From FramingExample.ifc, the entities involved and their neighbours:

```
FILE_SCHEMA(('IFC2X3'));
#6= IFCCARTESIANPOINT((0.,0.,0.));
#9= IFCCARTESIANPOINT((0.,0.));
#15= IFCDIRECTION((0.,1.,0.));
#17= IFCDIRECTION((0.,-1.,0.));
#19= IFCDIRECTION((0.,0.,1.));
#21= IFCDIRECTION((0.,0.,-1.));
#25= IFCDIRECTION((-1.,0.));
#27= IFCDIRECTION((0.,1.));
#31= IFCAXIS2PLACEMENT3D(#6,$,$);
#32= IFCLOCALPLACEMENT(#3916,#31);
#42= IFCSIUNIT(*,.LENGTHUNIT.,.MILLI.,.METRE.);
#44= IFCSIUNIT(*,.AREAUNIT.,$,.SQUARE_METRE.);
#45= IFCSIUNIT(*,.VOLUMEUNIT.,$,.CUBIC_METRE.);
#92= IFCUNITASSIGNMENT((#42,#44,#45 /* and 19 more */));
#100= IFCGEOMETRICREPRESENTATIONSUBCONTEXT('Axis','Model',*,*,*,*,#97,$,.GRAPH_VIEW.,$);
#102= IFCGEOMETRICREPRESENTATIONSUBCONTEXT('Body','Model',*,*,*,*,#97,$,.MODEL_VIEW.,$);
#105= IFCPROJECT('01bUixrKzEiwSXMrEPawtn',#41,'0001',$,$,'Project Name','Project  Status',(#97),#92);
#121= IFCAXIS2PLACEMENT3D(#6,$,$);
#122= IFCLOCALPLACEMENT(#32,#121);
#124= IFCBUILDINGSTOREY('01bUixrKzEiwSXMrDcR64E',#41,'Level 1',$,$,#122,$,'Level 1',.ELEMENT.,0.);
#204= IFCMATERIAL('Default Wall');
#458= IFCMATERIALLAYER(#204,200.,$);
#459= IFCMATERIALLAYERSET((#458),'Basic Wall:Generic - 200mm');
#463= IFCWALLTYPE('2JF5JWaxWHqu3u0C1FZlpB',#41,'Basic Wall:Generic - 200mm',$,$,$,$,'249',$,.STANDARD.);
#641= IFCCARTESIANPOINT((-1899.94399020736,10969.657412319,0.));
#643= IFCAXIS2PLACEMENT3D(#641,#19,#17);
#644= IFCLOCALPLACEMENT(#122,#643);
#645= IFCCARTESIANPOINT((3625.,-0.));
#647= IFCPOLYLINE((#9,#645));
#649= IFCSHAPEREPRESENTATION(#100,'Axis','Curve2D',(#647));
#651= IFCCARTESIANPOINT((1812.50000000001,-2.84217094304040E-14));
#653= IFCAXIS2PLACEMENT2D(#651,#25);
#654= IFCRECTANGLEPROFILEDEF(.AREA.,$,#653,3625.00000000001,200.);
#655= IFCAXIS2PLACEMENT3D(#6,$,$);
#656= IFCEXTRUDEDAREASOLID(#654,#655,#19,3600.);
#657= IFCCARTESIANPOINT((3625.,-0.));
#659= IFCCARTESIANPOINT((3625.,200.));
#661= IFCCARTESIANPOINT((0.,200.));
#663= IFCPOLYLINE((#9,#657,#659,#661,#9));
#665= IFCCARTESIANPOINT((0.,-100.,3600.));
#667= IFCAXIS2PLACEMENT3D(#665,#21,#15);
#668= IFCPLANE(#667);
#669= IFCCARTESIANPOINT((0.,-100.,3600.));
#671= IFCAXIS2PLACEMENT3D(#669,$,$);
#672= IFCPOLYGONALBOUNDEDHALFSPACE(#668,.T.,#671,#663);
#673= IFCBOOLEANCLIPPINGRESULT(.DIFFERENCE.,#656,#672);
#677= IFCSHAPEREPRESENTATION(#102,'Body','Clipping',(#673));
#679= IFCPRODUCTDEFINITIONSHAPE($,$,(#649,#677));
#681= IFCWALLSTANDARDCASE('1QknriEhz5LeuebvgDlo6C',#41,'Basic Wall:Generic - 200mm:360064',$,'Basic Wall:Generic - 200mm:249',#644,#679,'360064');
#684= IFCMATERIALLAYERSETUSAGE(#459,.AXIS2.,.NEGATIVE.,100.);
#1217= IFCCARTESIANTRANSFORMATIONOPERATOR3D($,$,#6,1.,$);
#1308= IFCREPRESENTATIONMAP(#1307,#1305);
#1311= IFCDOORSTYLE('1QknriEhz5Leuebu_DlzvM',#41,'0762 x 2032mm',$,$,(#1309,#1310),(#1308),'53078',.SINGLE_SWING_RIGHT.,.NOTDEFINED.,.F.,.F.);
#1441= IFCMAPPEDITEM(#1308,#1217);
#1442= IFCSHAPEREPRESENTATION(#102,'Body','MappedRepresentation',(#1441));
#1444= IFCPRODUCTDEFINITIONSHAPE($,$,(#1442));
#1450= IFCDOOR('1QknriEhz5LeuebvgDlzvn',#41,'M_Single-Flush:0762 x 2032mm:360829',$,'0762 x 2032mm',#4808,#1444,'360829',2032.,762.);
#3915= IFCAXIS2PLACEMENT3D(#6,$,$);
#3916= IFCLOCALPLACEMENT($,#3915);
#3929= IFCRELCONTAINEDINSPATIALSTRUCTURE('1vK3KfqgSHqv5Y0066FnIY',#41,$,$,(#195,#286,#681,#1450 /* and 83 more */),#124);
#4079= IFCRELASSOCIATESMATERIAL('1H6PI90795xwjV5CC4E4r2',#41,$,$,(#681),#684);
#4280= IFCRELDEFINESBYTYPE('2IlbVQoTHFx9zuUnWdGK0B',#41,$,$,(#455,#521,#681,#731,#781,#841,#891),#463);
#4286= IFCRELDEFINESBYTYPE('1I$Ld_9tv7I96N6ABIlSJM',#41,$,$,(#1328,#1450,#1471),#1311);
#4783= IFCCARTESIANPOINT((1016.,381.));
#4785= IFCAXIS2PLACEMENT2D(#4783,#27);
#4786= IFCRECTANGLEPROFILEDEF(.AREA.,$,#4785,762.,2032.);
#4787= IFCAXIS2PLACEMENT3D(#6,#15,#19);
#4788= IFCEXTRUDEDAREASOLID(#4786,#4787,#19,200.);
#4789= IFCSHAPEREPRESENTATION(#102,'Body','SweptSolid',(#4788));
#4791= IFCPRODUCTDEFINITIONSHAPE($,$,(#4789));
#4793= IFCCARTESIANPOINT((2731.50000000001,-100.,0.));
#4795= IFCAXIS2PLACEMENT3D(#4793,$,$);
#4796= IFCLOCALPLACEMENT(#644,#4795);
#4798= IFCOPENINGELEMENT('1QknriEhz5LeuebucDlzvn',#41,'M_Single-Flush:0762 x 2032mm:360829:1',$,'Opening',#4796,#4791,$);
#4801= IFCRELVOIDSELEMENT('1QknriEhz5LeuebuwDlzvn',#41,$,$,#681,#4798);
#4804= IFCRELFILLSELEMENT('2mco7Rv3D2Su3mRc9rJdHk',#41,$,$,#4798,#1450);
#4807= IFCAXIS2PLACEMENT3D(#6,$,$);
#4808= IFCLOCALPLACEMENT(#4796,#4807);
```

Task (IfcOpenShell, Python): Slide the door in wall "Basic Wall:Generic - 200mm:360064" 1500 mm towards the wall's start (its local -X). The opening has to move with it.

```python
import ifcopenshell
import ifcopenshell.api.geometry
import ifcopenshell.util.placement
import ifcopenshell.util.unit

model = ifcopenshell.open("FramingExample.ifc")
unit_scale = ifcopenshell.util.unit.calculate_unit_scale(model)

door = model.by_guid("1QknriEhz5LeuebvgDlzvn")
opening = door.FillsVoids[0].RelatingOpeningElement
wall = opening.VoidsElements[0].RelatingBuildingElement

wall_matrix = ifcopenshell.util.placement.get_local_placement(wall.ObjectPlacement)
shift = wall_matrix[:3, 0] * -1.5 / unit_scale
before = ifcopenshell.util.placement.get_local_placement(door.ObjectPlacement)[:3, 3].copy()

# The door is placed relative to its opening, so it follows when the opening moves.
matrix = ifcopenshell.util.placement.get_local_placement(opening.ObjectPlacement)
matrix[:3, 3] += shift
ifcopenshell.api.geometry.edit_object_placement(
    model, product=opening, matrix=matrix, is_si=False, should_transform_children=True
)

after = ifcopenshell.util.placement.get_local_placement(door.ObjectPlacement)[:3, 3]
print("door moved by", (after - before).round(3) + 0.0)

model.write("FramingExample_edited.ifc")
```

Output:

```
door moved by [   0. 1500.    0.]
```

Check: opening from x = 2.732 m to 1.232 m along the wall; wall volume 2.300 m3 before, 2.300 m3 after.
